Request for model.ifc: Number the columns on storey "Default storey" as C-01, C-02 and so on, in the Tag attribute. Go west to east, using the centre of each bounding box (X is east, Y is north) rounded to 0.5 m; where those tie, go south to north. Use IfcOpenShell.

First a look at what the model holds.

```python
import ifcopenshell
import ifcopenshell.util.element
import ifcopenshell.util.placement

model = ifcopenshell.open("model.ifc")
print(model.schema)
storey = next(s for s in model.by_type("IfcBuildingStorey") if s.Name == "Default storey")
columns = [e for e in ifcopenshell.util.element.get_decomposition(storey) if e.is_a("IfcColumn")]
for e in sorted(columns, key=lambda e: e.id()):
    origin = ifcopenshell.util.placement.get_local_placement(e.ObjectPlacement)[:3, 3]
    print(e.id(), e.Tag, e.Name, origin.round(2) + 0.0, sep=" | ")
```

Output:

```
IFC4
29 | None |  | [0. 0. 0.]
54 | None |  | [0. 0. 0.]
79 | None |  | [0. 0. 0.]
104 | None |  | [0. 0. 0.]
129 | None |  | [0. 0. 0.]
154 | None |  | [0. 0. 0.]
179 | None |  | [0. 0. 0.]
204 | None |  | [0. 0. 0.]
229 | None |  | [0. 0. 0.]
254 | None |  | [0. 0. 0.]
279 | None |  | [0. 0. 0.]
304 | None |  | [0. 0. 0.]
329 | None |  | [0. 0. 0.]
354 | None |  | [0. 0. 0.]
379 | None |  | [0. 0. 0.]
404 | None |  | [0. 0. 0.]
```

```python
import ifcopenshell
import ifcopenshell.geom
import ifcopenshell.util.element
import ifcopenshell.util.shape

model = ifcopenshell.open("model.ifc")
settings = ifcopenshell.geom.settings()
settings.set("use-world-coords", True)


def centre(element):
    shape = ifcopenshell.geom.create_shape(settings, element)
    return ifcopenshell.util.shape.get_bbox_centroid(shape.geometry)


storey = next(s for s in model.by_type("IfcBuildingStorey") if s.Name == "Default storey")
columns = [e for e in ifcopenshell.util.element.get_decomposition(storey) if e.is_a("IfcColumn")]

# Insertion points can sit at a corner or the storey origin, so sort by the geometry (in metres).
centres = {e: centre(e) for e in columns}
columns.sort(key=lambda e: (round(centres[e][0] / 0.5), centres[e][1]))

for i, e in enumerate(columns, start=1):
    number = f"C-{i:02d}"
    e.Tag = number
    print(e.id(), number)

model.write("model_rev.ifc")
```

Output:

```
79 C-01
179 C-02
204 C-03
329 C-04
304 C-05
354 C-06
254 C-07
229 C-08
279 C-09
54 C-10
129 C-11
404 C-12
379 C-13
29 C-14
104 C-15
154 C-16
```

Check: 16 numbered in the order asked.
